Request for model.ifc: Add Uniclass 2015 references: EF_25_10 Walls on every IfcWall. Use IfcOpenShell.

First a look at what the model holds.

```python
import ifcopenshell

model = ifcopenshell.open("model.ifc")
print(model.schema)
print("classifications:", [c.Name for c in model.by_type("IfcClassification")])
for ifc_class in ("IfcDoor", "IfcRoof", "IfcStair", "IfcWall", "IfcWindow"):
    print(ifc_class, len(model.by_type(ifc_class)))
```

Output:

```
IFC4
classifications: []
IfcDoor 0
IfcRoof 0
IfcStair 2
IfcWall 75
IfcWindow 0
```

```python
import ifcopenshell
import ifcopenshell.api.classification

model = ifcopenshell.open("model.ifc")

system = ifcopenshell.api.classification.add_classification(model, classification="Uniclass 2015")

codes = {
    "IfcWall": ("EF_25_10", "Walls"),
}
for ifc_class, (code, name) in codes.items():
    products = model.by_type(ifc_class)
    ifcopenshell.api.classification.add_reference(
        model, products=products, classification=system, identification=code, name=name
    )
    print(code, len(products))

model.write("model_updated.ifc")
```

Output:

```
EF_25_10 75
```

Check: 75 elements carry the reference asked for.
